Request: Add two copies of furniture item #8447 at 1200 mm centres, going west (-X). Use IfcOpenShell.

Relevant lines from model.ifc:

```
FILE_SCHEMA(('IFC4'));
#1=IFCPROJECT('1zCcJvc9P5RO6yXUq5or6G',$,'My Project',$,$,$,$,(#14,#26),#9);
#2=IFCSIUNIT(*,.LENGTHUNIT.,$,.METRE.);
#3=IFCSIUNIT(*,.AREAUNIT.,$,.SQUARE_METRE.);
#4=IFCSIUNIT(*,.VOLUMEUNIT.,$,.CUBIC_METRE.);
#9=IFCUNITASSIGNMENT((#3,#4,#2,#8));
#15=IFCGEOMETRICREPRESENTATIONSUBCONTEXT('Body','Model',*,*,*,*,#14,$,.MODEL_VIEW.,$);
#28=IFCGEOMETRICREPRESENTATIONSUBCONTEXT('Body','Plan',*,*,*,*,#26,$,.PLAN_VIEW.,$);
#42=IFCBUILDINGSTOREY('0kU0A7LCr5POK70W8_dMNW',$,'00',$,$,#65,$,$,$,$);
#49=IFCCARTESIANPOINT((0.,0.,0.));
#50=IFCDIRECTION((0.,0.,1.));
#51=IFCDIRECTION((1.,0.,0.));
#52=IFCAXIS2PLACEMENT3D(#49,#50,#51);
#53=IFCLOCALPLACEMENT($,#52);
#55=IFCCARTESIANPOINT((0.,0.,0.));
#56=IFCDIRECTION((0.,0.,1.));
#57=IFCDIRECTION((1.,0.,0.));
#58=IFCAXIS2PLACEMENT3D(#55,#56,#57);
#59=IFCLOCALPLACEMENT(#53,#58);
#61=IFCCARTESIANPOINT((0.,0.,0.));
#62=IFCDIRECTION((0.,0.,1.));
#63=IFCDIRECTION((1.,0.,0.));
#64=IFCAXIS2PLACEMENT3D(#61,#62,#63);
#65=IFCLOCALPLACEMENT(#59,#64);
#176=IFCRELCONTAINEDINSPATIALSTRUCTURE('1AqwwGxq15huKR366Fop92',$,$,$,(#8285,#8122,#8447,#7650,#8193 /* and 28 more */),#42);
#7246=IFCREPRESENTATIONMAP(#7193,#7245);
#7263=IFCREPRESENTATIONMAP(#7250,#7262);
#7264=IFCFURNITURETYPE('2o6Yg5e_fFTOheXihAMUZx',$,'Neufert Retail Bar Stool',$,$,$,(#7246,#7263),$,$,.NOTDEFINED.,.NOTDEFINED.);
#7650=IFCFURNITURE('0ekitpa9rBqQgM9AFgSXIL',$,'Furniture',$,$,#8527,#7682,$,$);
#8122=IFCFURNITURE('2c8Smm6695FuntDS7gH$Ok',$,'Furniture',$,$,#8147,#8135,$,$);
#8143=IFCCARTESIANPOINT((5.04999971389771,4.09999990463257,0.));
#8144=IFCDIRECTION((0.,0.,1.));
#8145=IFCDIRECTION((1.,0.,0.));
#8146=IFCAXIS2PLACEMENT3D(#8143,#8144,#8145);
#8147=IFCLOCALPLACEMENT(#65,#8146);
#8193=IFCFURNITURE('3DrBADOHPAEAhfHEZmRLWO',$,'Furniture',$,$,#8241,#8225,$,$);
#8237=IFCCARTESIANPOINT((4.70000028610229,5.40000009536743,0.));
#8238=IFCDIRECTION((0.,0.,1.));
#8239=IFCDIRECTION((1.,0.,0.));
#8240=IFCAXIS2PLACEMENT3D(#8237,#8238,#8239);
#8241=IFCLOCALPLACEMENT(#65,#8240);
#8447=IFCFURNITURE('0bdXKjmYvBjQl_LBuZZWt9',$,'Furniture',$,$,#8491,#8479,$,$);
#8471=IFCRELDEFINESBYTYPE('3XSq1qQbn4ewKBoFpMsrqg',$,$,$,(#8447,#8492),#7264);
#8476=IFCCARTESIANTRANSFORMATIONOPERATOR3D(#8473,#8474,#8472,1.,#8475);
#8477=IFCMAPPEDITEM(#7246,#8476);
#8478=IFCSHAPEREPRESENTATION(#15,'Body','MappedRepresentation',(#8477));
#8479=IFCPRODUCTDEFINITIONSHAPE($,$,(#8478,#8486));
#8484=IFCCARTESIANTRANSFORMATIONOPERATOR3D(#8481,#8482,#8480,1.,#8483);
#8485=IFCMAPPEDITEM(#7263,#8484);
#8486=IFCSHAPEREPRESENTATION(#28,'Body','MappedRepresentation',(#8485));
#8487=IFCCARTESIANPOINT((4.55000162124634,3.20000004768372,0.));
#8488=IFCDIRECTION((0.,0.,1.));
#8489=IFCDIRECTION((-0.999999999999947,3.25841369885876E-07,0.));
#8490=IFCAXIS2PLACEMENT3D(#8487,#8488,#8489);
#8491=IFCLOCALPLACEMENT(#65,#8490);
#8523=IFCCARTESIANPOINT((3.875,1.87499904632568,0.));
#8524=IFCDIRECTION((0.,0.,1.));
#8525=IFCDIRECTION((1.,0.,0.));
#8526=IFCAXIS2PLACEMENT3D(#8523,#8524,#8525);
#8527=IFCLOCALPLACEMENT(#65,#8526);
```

```python
import numpy as np
import ifcopenshell
import ifcopenshell.api.geometry
import ifcopenshell.api.root
import ifcopenshell.util.element
import ifcopenshell.util.placement
import ifcopenshell.util.unit

model = ifcopenshell.open("model.ifc")
unit_scale = ifcopenshell.util.unit.calculate_unit_scale(model)

source = model.by_guid("0bdXKjmYvBjQl_LBuZZWt9")
base = ifcopenshell.util.placement.get_local_placement(source.ObjectPlacement)
step = np.array([-1.0, 0.0, 0.0]) * 1.2 / unit_scale

for i in range(1, 3):
    copy = ifcopenshell.api.root.copy_class(model, product=source)
    copy.Representation = ifcopenshell.util.element.copy_deep(
        model, source.Representation, exclude=["IfcGeometricRepresentationContext", "IfcRepresentationMap"]
    )
    matrix = base.copy()
    matrix[:3, 3] += i * step
    print("added at", matrix[:3, 3].round(3) + 0.0)
    ifcopenshell.api.geometry.edit_object_placement(model, product=copy, matrix=matrix, is_si=False)

model.write("model_edited.ifc")
```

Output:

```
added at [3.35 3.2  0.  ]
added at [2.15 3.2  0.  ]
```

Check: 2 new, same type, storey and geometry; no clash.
